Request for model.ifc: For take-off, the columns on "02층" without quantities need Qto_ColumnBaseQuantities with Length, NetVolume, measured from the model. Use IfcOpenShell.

First a look at what the model holds.

```python
import ifcopenshell
import ifcopenshell.util.element
import ifcopenshell.util.unit

model = ifcopenshell.open("model.ifc")
print(model.schema)
for unit_type in ("LENGTHUNIT", "AREAUNIT", "VOLUMEUNIT"):
    print(unit_type, ifcopenshell.util.unit.calculate_unit_scale(model, unit_type))
storey = next(s for s in model.by_type("IfcBuildingStorey") if s.Name == "02층")
columns = [e for e in ifcopenshell.util.element.get_decomposition(storey) if e.is_a("IfcColumn")]
for e in sorted(columns, key=lambda e: e.id()):
    print(e.id(), e.is_a(), e.Name, list(ifcopenshell.util.element.get_psets(e, qtos_only=True)), sep=" | ")
```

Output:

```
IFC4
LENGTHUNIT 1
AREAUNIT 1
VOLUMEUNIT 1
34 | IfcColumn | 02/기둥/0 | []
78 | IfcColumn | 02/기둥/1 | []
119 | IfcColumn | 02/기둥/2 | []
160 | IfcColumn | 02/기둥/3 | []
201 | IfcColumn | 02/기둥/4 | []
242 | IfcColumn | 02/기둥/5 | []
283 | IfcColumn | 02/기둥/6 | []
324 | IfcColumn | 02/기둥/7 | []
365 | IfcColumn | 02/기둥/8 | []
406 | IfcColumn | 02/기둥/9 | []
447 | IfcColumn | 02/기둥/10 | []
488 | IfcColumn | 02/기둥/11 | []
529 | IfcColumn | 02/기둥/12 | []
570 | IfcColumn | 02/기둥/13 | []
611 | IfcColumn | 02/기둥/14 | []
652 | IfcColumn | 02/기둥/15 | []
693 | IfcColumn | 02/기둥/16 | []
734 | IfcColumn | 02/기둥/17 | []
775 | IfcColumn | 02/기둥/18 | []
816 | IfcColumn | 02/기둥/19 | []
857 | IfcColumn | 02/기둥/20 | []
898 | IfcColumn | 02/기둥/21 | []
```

```python
import ifcopenshell
import ifcopenshell.api.pset
import ifcopenshell.geom
import ifcopenshell.util.element
import ifcopenshell.util.shape
import ifcopenshell.util.unit

model = ifcopenshell.open("model.ifc")
unit_scale = ifcopenshell.util.unit.calculate_unit_scale(model)
volume_scale = ifcopenshell.util.unit.calculate_unit_scale(model, "VOLUMEUNIT")
settings = ifcopenshell.geom.settings()

storey = next(s for s in model.by_type("IfcBuildingStorey") if s.Name == "02층")
columns = [e for e in ifcopenshell.util.element.get_decomposition(storey) if e.is_a("IfcColumn")]

for e in sorted(columns, key=lambda e: e.id()):
    if ifcopenshell.util.element.get_psets(e, qtos_only=True, should_inherit=False):
        continue
    # Geometry comes back in metres, in the element's own axes.
    shape = ifcopenshell.geom.create_shape(settings, e)
    values = {
        "Length": ifcopenshell.util.shape.get_z(shape.geometry) / unit_scale,
        "NetVolume": ifcopenshell.util.shape.get_volume(shape.geometry) / volume_scale,
    }
    qto = ifcopenshell.api.pset.add_qto(model, product=e, name="Qto_ColumnBaseQuantities")
    ifcopenshell.api.pset.edit_qto(model, qto=qto, properties=values)
    print(e.id(), {k: round(v, 3) for k, v in values.items()})

model.write("model_edited.ifc")
```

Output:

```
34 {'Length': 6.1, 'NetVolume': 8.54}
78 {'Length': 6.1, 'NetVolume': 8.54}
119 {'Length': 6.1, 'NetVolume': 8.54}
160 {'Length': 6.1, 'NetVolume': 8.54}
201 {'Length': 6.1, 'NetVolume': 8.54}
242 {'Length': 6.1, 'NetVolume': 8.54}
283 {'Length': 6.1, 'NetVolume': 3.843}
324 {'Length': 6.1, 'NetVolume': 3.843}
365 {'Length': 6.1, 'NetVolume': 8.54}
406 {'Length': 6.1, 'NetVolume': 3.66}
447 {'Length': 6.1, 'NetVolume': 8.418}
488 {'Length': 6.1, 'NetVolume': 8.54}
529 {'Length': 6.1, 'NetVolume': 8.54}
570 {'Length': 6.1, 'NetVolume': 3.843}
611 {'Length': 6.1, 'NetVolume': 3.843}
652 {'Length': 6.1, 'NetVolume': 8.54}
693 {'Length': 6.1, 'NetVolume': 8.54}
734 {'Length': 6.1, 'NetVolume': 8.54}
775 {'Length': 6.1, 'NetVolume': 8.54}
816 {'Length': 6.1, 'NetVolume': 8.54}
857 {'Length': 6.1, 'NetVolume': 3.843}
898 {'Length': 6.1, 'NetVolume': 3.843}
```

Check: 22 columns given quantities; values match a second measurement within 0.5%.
